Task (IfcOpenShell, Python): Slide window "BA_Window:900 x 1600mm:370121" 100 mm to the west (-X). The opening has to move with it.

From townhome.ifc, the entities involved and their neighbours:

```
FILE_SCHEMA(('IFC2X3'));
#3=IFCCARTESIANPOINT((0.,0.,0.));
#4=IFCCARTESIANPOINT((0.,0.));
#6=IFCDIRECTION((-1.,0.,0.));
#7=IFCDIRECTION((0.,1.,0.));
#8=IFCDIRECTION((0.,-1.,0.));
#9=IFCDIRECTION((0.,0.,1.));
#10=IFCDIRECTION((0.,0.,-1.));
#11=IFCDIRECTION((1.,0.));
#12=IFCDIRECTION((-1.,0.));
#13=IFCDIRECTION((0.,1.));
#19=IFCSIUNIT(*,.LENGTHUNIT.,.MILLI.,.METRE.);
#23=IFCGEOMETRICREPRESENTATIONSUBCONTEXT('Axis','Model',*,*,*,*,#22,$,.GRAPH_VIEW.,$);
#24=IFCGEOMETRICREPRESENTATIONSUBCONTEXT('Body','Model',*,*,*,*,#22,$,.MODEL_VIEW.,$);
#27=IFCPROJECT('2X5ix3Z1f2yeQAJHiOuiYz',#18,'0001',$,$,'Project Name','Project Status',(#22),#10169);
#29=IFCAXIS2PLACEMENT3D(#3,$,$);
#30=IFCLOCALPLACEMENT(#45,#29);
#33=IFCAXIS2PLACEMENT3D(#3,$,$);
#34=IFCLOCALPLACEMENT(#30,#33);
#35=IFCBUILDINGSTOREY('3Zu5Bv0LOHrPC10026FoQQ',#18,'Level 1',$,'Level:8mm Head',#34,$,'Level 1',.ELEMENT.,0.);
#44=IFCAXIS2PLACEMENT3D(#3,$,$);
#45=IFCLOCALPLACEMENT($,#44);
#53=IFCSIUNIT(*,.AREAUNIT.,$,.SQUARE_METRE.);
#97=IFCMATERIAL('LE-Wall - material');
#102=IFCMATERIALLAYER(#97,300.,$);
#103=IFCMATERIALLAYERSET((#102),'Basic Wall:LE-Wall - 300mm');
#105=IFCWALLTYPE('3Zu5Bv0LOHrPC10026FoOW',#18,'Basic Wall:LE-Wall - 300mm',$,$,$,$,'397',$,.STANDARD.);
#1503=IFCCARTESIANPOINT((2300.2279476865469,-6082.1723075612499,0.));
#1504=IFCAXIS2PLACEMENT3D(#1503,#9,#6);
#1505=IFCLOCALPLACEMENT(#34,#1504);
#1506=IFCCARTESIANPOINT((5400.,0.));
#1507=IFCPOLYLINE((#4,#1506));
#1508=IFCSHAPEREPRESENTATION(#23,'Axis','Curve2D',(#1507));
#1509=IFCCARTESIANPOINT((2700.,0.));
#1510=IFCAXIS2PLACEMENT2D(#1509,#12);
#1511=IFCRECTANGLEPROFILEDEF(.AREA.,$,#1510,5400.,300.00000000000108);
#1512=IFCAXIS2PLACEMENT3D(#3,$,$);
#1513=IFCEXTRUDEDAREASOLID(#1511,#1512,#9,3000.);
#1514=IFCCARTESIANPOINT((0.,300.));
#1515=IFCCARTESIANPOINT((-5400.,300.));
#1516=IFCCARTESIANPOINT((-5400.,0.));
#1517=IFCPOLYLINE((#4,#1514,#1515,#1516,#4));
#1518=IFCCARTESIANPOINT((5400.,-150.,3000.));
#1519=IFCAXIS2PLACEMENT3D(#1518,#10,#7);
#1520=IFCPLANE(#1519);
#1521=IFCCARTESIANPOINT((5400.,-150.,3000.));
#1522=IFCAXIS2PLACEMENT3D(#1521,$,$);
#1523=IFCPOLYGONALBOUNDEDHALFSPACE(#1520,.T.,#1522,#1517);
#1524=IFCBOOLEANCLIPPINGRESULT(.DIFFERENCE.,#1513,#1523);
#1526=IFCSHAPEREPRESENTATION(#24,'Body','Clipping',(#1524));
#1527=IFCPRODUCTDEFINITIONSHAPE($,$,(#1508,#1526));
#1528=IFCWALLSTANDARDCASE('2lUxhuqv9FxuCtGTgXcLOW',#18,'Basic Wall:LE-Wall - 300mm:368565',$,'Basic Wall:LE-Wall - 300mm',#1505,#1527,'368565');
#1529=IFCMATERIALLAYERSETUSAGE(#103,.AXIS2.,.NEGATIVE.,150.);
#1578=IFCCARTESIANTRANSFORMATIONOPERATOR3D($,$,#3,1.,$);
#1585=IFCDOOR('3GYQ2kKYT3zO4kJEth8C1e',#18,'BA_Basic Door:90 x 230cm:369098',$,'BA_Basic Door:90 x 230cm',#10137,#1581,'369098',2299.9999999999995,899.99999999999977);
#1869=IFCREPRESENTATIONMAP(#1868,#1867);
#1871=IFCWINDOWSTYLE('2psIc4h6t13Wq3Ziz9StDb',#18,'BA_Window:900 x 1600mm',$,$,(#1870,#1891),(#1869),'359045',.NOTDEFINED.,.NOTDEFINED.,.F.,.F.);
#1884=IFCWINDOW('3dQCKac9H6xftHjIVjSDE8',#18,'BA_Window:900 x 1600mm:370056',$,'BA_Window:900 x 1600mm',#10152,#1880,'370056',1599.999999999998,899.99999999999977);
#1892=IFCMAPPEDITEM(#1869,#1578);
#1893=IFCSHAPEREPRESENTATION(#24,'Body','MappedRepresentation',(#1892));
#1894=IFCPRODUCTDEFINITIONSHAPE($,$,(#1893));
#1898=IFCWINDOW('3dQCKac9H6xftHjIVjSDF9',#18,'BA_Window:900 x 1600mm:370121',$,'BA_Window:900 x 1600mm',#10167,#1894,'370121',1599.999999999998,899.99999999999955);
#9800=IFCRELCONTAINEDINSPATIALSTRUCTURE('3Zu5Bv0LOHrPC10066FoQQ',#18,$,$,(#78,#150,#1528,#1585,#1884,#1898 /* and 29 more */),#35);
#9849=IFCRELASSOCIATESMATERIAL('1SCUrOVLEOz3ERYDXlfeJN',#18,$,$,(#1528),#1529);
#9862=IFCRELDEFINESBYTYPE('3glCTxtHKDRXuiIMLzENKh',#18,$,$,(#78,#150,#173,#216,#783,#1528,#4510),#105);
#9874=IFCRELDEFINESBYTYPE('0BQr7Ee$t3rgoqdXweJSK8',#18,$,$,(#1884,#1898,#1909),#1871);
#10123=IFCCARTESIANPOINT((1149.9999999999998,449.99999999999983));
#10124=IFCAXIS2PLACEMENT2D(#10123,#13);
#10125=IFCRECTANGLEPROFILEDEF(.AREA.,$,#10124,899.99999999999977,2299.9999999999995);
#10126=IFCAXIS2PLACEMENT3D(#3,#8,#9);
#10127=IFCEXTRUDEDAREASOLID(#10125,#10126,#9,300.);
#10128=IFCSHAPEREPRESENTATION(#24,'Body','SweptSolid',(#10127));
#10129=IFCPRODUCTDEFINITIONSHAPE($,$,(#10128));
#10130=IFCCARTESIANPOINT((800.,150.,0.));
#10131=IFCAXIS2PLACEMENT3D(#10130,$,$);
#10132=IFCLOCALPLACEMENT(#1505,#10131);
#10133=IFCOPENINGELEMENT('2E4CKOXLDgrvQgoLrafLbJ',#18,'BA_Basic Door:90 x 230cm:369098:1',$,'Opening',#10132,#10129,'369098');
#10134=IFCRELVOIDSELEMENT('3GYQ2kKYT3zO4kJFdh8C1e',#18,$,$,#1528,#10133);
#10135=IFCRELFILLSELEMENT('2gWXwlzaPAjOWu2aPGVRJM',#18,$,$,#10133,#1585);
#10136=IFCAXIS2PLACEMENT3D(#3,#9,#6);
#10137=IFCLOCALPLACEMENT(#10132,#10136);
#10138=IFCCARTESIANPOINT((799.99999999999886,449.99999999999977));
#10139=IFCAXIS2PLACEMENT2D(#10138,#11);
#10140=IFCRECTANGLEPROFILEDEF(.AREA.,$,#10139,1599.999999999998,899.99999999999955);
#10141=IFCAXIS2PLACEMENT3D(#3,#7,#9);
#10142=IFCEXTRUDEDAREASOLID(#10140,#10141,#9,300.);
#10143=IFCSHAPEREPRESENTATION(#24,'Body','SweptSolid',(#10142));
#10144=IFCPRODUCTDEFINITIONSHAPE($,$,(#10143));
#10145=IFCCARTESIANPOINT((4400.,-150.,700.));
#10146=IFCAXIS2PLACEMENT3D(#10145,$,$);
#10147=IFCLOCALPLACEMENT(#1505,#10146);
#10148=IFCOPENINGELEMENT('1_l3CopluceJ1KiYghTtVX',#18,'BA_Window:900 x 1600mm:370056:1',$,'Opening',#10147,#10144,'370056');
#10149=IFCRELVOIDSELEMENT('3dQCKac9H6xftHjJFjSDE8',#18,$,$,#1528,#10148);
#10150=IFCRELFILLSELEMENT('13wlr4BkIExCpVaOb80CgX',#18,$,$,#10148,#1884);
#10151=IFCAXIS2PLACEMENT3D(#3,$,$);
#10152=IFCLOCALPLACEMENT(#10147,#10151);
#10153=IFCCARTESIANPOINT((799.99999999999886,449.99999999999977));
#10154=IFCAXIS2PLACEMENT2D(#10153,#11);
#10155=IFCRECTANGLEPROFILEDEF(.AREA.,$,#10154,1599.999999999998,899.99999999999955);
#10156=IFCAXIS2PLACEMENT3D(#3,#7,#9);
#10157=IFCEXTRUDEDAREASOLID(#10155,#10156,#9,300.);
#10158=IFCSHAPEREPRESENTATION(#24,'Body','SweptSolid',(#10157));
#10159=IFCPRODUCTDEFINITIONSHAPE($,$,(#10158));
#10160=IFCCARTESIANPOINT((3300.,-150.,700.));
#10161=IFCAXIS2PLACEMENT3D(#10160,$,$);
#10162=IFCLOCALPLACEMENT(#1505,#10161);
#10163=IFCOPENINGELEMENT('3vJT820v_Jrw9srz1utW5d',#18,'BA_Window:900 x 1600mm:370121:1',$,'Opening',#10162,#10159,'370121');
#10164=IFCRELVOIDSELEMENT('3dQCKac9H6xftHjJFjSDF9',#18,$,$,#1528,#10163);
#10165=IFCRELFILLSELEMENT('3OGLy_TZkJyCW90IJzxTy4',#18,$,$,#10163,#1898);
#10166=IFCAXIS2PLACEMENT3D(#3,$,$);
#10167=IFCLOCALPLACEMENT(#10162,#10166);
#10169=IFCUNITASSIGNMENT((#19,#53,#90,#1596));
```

```python
import ifcopenshell
import ifcopenshell.api.geometry
import ifcopenshell.util.placement
import ifcopenshell.util.unit

model = ifcopenshell.open("townhome.ifc")
unit_scale = ifcopenshell.util.unit.calculate_unit_scale(model)

window = model.by_guid("3dQCKac9H6xftHjIVjSDF9")
opening = window.FillsVoids[0].RelatingOpeningElement
wall = opening.VoidsElements[0].RelatingBuildingElement

wall_matrix = ifcopenshell.util.placement.get_local_placement(wall.ObjectPlacement)
shift = wall_matrix[:3, 0] * 0.1 / unit_scale
before = ifcopenshell.util.placement.get_local_placement(window.ObjectPlacement)[:3, 3].copy()

# The window is placed relative to its opening, so it follows when the opening moves.
matrix = ifcopenshell.util.placement.get_local_placement(opening.ObjectPlacement)
matrix[:3, 3] += shift
ifcopenshell.api.geometry.edit_object_placement(
    model, product=opening, matrix=matrix, is_si=False, should_transform_children=True
)

after = ifcopenshell.util.placement.get_local_placement(window.ObjectPlacement)[:3, 3]
print("window moved by", (after - before).round(3) + 0.0)

model.write("townhome_v2.ifc")
```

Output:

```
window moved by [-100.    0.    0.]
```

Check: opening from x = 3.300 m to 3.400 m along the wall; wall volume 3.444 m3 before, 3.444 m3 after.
